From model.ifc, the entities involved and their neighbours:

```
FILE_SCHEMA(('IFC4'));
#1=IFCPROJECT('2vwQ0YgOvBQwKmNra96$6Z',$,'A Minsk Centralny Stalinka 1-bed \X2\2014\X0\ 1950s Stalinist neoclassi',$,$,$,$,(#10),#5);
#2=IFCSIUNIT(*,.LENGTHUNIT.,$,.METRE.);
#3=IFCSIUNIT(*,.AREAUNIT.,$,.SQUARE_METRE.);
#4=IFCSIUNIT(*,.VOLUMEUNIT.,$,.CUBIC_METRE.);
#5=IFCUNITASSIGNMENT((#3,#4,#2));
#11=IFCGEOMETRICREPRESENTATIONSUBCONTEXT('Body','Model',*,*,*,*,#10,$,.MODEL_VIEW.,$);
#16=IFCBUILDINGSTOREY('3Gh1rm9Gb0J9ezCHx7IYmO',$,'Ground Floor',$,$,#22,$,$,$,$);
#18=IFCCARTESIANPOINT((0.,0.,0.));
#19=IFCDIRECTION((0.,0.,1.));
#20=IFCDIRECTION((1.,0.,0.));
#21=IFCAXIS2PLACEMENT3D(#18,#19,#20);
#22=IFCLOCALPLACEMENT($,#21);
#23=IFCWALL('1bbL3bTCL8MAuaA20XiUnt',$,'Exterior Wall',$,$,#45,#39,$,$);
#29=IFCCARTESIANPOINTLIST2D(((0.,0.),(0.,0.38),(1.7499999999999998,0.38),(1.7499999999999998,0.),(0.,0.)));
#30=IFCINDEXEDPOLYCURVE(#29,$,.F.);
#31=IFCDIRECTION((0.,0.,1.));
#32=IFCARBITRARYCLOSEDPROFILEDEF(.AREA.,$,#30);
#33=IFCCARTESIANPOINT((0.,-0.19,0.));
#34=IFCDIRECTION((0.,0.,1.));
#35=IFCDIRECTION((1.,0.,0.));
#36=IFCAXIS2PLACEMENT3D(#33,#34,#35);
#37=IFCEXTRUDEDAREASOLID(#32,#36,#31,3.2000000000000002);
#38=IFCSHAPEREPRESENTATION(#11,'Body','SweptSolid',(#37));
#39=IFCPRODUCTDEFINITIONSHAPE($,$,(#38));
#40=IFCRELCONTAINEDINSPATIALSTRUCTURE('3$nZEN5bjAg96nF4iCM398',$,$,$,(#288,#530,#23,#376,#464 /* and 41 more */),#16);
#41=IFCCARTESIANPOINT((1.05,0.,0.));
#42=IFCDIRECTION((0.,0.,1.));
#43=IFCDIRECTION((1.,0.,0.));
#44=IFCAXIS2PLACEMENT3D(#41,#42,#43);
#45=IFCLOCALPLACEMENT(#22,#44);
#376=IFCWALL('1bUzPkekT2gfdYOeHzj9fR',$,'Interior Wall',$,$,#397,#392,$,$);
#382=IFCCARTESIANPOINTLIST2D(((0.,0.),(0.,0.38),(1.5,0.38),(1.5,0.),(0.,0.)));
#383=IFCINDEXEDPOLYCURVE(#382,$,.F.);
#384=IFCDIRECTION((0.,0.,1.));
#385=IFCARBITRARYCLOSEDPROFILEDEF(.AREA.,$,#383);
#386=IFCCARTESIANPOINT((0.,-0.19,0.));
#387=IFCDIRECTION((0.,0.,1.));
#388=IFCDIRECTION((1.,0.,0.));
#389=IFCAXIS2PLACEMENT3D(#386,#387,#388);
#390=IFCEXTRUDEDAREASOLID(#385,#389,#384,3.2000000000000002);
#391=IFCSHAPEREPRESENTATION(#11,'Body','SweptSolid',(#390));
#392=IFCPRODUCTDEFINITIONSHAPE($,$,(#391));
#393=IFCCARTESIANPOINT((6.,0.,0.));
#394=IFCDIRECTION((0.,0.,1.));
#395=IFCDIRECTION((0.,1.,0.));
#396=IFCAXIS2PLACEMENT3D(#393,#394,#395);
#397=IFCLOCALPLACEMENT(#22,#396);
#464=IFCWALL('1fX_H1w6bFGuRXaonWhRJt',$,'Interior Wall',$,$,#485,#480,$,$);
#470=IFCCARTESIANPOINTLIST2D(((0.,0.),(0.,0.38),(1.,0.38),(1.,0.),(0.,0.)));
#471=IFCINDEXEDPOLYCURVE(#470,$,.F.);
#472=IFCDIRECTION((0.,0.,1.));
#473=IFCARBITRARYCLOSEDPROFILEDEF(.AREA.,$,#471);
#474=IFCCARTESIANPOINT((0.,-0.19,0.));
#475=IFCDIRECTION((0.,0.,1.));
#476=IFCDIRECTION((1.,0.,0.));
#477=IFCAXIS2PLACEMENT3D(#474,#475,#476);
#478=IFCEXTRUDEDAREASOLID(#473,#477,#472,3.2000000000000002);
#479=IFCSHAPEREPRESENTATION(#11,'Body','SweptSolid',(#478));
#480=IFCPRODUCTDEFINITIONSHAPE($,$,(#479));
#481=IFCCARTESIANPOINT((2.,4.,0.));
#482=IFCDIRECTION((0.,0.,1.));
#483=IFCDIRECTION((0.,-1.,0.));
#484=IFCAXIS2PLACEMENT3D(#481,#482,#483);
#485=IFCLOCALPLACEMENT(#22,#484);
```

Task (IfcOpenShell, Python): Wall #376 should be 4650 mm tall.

```python
import ifcopenshell
import ifcopenshell.geom
import ifcopenshell.util.representation
import ifcopenshell.util.shape
import ifcopenshell.util.unit

model = ifcopenshell.open("model.ifc")
unit_scale = ifcopenshell.util.unit.calculate_unit_scale(model)
settings = ifcopenshell.geom.settings()


def volume(element):
    """Net volume in cubic metres, openings subtracted."""
    shape = ifcopenshell.geom.create_shape(settings, element)
    return ifcopenshell.util.shape.get_volume(shape.geometry)


wall = model.by_guid("1bUzPkekT2gfdYOeHzj9fR")
before = volume(wall)

body = ifcopenshell.util.representation.get_representation(wall, "Model", "Body")
solid = body.Items[0]
old_height = solid.Depth
solid.Depth = 4.65 / unit_scale
after = volume(wall)

print(f"height {old_height:g} -> {solid.Depth:g}, volume {before:.3f} -> {after:.3f} m3")

model.write("model_v2.ifc")
```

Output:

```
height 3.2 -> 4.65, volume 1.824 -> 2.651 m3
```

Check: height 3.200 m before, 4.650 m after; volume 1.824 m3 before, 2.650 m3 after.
